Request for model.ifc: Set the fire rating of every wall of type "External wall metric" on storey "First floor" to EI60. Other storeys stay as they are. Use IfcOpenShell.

First a look at what the model holds.

```python
import ifcopenshell
import ifcopenshell.util.element

model = ifcopenshell.open("model.ifc")
print(model.schema)
storey = next(s for s in model.by_type("IfcBuildingStorey") if s.Name == "First floor")
walls = [e for e in ifcopenshell.util.element.get_decomposition(storey) if e.is_a("IfcWall")]
seen = {}
for e in walls:
    element_type = ifcopenshell.util.element.get_type(e)
    key = (element_type.Name if element_type != e and element_type else None, ifcopenshell.util.element.get_pset(e, "Pset_WallCommon", "FireRating"))
    seen[key] = seen.get(key, 0) + 1
for (name, value), count in sorted(seen.items(), key=str):
    print(count, "x", name, "|", value)
```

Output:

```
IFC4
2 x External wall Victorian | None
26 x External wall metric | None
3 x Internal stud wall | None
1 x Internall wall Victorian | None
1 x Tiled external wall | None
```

```python
import ifcopenshell
import ifcopenshell.api.pset
import ifcopenshell.util.element

model = ifcopenshell.open("model.ifc")

storey = next(s for s in model.by_type("IfcBuildingStorey") if s.Name == "First floor")
walls = [e for e in ifcopenshell.util.element.get_decomposition(storey) if e.is_a("IfcWall")]

count = 0
for e in walls:
    element_type = ifcopenshell.util.element.get_type(e)
    if element_type in (None, e) or element_type.Name != "External wall metric":
        continue
    # add_pset returns the element's existing set when there is one.
    pset = ifcopenshell.api.pset.add_pset(model, product=e, name="Pset_WallCommon")
    ifcopenshell.api.pset.edit_pset(model, pset=pset, properties={"FireRating": "EI60"})
    count += 1

print(count, "walls updated")

model.write("model_v2.ifc")
```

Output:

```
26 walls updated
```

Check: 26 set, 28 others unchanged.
